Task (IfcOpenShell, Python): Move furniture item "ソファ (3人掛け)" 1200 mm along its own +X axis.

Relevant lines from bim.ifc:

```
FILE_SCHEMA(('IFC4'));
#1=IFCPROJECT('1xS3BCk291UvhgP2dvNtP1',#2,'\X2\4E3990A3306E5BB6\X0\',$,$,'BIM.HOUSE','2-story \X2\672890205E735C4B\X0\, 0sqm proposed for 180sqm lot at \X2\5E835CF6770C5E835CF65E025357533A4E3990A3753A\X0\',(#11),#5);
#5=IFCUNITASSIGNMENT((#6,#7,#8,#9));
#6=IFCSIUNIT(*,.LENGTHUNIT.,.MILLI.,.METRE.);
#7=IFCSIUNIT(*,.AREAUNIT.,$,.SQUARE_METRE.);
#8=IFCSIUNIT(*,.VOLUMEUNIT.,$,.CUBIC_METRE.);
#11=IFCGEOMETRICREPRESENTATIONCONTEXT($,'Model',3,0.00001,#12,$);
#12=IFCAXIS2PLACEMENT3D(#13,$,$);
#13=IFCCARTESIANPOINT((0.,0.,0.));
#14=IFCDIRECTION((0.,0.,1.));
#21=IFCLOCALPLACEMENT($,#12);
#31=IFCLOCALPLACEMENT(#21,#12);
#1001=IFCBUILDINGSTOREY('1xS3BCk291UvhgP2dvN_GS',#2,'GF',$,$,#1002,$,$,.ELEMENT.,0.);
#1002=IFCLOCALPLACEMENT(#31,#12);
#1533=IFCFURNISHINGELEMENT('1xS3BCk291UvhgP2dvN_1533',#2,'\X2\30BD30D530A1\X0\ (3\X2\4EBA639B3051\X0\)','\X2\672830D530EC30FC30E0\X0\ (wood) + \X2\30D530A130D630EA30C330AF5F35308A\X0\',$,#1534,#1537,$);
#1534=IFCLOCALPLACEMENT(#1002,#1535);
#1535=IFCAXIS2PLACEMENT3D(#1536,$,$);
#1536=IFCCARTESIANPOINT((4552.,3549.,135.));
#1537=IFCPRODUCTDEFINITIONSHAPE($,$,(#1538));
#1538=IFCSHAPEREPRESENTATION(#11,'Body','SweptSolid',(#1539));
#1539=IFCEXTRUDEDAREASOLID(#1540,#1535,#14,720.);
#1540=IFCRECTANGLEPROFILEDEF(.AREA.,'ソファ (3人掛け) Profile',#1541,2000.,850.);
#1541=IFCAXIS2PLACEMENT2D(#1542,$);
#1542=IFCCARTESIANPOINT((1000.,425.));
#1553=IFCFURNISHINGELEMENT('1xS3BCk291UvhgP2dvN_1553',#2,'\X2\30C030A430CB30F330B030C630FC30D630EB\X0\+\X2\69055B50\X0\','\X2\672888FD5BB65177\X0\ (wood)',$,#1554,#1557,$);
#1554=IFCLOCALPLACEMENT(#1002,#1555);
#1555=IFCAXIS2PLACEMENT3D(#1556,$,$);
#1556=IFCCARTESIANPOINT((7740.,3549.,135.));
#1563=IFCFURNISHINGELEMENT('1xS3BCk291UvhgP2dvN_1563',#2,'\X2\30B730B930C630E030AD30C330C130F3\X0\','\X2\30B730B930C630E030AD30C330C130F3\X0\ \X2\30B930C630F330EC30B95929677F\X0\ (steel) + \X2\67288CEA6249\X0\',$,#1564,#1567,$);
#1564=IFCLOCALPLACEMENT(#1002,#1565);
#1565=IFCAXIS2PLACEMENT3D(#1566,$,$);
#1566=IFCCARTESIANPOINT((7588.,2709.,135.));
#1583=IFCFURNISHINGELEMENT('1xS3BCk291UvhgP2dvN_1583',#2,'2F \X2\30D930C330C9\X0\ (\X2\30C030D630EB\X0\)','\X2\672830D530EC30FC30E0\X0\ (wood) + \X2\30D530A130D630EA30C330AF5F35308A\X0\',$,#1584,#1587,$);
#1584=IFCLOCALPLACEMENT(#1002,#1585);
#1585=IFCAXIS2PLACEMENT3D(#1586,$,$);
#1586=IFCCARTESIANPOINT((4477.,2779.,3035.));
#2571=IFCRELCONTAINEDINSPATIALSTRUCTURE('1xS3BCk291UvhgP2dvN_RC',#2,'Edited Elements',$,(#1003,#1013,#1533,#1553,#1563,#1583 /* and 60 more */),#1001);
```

```python
import ifcopenshell
import ifcopenshell.api.geometry
import ifcopenshell.util.placement
import ifcopenshell.util.unit

model = ifcopenshell.open("bim.ifc")
unit_scale = ifcopenshell.util.unit.calculate_unit_scale(model)

item = model.by_guid("1xS3BCk291UvhgP2dvN_1533")
matrix = ifcopenshell.util.placement.get_local_placement(item.ObjectPlacement)
matrix[:3, 3] += matrix[:3, 0] * 1.2 / unit_scale
ifcopenshell.api.geometry.edit_object_placement(model, product=item, matrix=matrix, is_si=False)

print(ifcopenshell.util.placement.get_local_placement(item.ObjectPlacement).round(3) + 0.0)

model.write("bim_v2.ifc")
```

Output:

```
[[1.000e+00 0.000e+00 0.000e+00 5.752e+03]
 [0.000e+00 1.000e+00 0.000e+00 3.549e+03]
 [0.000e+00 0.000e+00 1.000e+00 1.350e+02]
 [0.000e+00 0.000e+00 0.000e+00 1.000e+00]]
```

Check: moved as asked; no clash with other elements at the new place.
